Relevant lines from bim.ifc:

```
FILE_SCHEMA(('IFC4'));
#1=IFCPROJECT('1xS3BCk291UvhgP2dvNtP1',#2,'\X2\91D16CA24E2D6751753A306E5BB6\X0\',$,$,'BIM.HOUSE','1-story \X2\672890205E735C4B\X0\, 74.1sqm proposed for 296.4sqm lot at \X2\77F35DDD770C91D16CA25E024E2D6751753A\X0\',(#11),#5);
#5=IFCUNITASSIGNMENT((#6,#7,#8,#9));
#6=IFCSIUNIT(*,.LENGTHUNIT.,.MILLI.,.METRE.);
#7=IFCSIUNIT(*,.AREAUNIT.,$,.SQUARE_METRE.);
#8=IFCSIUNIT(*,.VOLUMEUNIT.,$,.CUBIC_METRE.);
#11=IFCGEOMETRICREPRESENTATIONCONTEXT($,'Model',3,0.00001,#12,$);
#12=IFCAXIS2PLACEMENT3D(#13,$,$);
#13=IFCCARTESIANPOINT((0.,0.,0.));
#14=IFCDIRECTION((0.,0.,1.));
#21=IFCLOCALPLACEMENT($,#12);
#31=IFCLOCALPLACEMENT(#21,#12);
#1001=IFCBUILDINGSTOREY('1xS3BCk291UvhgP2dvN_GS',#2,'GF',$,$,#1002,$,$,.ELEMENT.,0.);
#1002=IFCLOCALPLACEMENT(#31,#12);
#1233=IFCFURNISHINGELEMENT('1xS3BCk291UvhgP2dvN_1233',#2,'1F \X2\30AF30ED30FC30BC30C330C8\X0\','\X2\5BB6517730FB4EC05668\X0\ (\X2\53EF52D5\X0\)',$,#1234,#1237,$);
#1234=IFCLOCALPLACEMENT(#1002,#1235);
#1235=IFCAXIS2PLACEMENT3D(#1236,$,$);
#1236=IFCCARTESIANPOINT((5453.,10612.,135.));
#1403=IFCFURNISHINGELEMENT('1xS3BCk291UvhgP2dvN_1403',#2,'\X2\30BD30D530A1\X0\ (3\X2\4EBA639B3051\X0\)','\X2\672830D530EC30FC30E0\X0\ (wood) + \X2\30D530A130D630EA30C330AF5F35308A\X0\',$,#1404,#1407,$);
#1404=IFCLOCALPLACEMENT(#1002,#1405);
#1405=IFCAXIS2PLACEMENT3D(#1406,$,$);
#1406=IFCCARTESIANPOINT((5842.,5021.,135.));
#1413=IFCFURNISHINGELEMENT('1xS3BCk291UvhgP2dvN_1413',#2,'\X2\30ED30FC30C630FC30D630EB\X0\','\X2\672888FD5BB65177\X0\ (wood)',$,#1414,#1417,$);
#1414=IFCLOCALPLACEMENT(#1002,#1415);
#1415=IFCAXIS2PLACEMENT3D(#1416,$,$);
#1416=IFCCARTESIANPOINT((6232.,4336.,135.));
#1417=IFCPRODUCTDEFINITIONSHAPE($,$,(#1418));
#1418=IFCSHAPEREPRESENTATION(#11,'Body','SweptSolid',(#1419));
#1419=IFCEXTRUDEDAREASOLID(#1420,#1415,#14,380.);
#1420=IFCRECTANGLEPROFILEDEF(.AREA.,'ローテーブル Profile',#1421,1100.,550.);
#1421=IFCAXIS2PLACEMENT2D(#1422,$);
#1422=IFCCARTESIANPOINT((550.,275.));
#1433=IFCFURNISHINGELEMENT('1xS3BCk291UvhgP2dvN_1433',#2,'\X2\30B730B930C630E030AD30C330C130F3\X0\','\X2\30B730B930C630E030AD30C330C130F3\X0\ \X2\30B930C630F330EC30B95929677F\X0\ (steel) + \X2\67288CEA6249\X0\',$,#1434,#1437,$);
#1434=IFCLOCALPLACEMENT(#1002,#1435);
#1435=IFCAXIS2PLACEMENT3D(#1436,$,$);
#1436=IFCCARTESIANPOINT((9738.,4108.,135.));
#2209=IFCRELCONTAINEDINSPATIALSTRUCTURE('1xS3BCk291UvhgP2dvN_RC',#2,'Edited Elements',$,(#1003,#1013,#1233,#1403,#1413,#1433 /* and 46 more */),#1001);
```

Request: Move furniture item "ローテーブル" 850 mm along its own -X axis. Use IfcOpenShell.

```python
import ifcopenshell
import ifcopenshell.api.geometry
import ifcopenshell.util.placement
import ifcopenshell.util.unit

model = ifcopenshell.open("bim.ifc")
unit_scale = ifcopenshell.util.unit.calculate_unit_scale(model)

item = model.by_guid("1xS3BCk291UvhgP2dvN_1413")
matrix = ifcopenshell.util.placement.get_local_placement(item.ObjectPlacement)
matrix[:3, 3] -= matrix[:3, 0] * 0.85 / unit_scale
ifcopenshell.api.geometry.edit_object_placement(model, product=item, matrix=matrix, is_si=False)

print(ifcopenshell.util.placement.get_local_placement(item.ObjectPlacement).round(3) + 0.0)

model.write("bim_edited.ifc")
```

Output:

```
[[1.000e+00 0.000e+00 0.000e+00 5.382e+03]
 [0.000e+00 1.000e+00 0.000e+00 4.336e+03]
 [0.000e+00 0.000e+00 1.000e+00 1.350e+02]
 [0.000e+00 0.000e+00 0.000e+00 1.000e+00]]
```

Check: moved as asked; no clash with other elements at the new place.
